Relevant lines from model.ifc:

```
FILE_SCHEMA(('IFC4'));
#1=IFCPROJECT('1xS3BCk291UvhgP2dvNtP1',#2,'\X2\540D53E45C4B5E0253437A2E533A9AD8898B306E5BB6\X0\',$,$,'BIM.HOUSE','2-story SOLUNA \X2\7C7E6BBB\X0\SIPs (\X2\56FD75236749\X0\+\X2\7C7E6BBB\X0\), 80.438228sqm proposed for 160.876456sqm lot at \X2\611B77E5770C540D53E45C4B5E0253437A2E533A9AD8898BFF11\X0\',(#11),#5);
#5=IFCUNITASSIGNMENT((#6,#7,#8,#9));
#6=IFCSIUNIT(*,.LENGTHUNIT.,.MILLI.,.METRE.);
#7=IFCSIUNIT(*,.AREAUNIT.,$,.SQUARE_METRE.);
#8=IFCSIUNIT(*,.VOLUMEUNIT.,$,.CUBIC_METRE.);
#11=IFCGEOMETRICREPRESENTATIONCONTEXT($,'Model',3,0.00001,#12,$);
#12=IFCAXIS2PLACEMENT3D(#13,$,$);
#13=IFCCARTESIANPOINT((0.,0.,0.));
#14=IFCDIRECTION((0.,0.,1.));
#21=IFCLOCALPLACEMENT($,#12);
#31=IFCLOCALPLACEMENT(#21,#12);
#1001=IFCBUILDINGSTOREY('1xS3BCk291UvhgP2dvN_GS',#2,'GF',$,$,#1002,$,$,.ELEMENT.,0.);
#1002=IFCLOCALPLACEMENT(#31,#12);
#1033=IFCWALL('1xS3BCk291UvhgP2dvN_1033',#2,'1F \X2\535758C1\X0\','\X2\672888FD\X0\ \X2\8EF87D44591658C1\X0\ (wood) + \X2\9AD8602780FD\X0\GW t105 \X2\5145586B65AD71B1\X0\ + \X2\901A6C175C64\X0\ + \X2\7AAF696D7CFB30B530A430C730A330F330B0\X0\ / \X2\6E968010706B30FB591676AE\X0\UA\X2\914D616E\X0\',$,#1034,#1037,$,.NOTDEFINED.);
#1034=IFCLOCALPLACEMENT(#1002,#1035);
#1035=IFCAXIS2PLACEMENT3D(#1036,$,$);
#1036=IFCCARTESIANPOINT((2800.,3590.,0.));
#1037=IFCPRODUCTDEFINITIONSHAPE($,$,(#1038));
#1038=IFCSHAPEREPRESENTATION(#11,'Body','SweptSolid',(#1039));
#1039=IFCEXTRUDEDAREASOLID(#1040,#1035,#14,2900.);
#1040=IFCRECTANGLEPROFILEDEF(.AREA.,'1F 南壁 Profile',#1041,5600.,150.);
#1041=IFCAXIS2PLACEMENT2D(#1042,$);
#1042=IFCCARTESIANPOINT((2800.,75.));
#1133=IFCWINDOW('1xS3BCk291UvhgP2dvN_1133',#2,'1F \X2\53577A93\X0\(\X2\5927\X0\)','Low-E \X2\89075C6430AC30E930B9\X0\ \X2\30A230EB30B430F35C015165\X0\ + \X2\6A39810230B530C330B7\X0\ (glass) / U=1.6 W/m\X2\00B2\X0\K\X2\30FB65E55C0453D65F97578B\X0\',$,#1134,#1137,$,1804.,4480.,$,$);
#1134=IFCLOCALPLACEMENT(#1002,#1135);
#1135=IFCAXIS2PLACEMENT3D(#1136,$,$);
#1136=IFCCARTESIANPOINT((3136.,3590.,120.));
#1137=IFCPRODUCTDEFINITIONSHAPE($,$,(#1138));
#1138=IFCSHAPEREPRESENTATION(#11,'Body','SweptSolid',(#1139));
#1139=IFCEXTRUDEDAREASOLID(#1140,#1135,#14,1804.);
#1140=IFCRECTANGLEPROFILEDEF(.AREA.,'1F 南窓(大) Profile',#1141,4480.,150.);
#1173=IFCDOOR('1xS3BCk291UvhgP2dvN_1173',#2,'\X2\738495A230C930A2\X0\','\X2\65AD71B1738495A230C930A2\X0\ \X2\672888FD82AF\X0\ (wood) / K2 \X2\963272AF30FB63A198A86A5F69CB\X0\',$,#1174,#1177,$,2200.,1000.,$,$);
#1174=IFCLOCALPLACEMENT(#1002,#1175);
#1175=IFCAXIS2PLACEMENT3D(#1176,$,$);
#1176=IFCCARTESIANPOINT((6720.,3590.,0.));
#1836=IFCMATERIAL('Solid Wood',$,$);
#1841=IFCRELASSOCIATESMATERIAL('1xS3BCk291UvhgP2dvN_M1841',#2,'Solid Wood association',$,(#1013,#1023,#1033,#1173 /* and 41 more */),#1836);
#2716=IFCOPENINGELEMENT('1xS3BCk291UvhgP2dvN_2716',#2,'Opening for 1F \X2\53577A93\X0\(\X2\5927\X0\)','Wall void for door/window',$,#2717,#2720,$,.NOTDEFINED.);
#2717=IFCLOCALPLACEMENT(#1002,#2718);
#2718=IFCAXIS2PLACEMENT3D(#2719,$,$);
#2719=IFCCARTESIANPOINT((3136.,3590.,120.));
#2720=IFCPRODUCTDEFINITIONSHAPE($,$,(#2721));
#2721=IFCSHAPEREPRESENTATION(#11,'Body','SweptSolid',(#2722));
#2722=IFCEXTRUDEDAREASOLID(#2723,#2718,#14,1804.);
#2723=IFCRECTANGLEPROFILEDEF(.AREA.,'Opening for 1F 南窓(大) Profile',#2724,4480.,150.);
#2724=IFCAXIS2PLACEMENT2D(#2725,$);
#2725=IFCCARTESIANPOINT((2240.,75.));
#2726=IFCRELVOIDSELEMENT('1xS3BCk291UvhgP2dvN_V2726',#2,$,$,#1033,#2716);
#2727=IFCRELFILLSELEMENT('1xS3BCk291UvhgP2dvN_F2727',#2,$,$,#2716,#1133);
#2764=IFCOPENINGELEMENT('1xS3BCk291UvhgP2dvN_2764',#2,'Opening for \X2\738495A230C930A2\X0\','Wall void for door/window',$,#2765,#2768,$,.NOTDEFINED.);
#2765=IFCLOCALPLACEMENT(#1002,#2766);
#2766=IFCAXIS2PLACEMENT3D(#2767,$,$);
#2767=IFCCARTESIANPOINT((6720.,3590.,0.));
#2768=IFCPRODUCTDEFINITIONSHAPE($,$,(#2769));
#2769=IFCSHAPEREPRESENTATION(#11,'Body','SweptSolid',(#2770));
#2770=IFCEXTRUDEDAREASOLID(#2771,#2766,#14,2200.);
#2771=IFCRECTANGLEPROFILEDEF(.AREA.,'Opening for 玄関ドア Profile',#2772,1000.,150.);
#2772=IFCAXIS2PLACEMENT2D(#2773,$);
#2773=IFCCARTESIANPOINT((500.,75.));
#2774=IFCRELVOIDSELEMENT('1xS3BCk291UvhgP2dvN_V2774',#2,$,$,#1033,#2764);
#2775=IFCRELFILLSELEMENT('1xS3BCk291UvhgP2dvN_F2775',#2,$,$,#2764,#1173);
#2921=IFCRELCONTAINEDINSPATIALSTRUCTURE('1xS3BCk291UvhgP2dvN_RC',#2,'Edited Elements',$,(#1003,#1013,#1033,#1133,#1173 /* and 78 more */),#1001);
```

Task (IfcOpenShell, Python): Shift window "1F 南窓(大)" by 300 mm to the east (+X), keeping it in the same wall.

```python
import ifcopenshell
import ifcopenshell.api.geometry
import ifcopenshell.util.placement
import ifcopenshell.util.unit

model = ifcopenshell.open("model.ifc")
unit_scale = ifcopenshell.util.unit.calculate_unit_scale(model)

window = model.by_guid("1xS3BCk291UvhgP2dvN_1133")
opening = window.FillsVoids[0].RelatingOpeningElement
wall = opening.VoidsElements[0].RelatingBuildingElement

wall_matrix = ifcopenshell.util.placement.get_local_placement(wall.ObjectPlacement)
shift = wall_matrix[:3, 0] * 0.3 / unit_scale
before = ifcopenshell.util.placement.get_local_placement(window.ObjectPlacement)[:3, 3].copy()

# The window is not placed relative to its opening, so move both.
for product in (opening, window):
    matrix = ifcopenshell.util.placement.get_local_placement(product.ObjectPlacement)
    matrix[:3, 3] += shift
    ifcopenshell.api.geometry.edit_object_placement(model, product=product, matrix=matrix, is_si=False)

after = ifcopenshell.util.placement.get_local_placement(window.ObjectPlacement)[:3, 3]
print("window moved by", (after - before).round(3) + 0.0)

model.write("model_v2.ifc")
```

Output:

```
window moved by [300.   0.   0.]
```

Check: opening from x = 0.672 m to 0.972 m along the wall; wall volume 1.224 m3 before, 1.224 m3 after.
